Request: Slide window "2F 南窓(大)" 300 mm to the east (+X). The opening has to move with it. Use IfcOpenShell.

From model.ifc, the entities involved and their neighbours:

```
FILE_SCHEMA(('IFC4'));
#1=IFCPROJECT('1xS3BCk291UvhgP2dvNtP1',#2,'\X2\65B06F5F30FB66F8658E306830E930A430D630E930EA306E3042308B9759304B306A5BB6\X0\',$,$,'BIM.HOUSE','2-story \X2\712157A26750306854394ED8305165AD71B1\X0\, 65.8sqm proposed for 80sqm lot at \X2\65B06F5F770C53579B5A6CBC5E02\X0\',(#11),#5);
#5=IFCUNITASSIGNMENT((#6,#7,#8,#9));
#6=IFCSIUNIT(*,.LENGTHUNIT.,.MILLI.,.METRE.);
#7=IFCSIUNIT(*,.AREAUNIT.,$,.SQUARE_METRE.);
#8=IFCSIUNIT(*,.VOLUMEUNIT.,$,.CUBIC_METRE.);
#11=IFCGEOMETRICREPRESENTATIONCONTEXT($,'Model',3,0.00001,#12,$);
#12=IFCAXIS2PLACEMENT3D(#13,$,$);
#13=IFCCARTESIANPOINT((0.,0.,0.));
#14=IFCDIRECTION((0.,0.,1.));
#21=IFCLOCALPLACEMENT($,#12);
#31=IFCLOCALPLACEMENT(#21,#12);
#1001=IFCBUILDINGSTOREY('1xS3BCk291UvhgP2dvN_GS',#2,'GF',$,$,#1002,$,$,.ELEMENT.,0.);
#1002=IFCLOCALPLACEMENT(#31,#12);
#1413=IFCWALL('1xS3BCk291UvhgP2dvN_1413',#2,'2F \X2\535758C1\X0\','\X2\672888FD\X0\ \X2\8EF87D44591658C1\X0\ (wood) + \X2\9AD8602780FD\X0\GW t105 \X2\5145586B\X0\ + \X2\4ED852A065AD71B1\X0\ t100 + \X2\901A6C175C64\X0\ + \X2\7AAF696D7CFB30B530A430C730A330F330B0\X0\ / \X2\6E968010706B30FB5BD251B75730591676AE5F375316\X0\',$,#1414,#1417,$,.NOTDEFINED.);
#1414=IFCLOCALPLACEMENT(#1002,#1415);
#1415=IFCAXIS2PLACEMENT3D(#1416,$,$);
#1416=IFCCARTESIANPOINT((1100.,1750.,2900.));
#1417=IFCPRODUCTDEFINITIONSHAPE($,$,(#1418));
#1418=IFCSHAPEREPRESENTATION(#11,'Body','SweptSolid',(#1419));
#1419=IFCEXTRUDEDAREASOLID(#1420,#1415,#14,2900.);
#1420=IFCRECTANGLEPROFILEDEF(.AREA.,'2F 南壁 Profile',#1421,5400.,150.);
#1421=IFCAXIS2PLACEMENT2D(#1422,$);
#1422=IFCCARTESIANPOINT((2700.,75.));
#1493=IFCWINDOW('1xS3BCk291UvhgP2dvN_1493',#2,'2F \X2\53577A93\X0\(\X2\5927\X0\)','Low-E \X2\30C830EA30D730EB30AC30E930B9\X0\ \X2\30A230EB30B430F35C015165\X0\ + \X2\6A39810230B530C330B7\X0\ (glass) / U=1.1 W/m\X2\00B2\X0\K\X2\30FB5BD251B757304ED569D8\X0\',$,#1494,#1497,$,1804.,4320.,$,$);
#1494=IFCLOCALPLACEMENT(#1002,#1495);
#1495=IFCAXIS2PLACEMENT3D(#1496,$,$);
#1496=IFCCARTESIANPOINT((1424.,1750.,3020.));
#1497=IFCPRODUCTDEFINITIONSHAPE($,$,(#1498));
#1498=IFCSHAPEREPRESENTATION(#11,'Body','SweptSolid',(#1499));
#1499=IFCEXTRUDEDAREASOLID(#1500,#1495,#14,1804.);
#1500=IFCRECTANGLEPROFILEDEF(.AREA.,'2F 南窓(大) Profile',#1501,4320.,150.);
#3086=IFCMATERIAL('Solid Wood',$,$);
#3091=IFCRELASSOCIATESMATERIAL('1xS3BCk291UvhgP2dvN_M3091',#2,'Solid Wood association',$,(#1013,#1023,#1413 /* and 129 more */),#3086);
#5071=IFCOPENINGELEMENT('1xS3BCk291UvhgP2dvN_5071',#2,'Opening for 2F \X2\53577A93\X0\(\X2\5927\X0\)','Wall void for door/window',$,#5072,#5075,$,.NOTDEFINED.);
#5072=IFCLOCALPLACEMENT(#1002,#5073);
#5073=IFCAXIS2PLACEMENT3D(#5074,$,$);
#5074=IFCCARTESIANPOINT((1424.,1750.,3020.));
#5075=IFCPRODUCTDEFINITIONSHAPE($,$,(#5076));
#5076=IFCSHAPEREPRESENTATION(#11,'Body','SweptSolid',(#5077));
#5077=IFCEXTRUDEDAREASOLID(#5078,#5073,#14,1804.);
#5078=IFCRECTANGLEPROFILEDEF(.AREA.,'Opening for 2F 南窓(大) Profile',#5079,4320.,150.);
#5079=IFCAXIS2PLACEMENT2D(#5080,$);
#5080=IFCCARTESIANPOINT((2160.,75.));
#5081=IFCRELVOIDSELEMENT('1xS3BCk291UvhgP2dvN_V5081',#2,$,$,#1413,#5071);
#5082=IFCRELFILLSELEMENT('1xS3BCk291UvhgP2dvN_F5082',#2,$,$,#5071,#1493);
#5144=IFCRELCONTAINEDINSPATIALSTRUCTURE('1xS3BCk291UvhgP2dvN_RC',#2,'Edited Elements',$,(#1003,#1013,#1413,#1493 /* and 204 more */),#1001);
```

```python
import ifcopenshell
import ifcopenshell.api.geometry
import ifcopenshell.util.placement
import ifcopenshell.util.unit

model = ifcopenshell.open("model.ifc")
unit_scale = ifcopenshell.util.unit.calculate_unit_scale(model)

window = model.by_id(1493)
opening = window.FillsVoids[0].RelatingOpeningElement
wall = opening.VoidsElements[0].RelatingBuildingElement

wall_matrix = ifcopenshell.util.placement.get_local_placement(wall.ObjectPlacement)
shift = wall_matrix[:3, 0] * 0.3 / unit_scale
before = ifcopenshell.util.placement.get_local_placement(window.ObjectPlacement)[:3, 3].copy()

# The window is not placed relative to its opening, so move both.
for product in (opening, window):
    matrix = ifcopenshell.util.placement.get_local_placement(product.ObjectPlacement)
    matrix[:3, 3] += shift
    ifcopenshell.api.geometry.edit_object_placement(model, product=product, matrix=matrix, is_si=False)

after = ifcopenshell.util.placement.get_local_placement(window.ObjectPlacement)[:3, 3]
print("window moved by", (after - before).round(3) + 0.0)

model.write("model_edited.ifc")
```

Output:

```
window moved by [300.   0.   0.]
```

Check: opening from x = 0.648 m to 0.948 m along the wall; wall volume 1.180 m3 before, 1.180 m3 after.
